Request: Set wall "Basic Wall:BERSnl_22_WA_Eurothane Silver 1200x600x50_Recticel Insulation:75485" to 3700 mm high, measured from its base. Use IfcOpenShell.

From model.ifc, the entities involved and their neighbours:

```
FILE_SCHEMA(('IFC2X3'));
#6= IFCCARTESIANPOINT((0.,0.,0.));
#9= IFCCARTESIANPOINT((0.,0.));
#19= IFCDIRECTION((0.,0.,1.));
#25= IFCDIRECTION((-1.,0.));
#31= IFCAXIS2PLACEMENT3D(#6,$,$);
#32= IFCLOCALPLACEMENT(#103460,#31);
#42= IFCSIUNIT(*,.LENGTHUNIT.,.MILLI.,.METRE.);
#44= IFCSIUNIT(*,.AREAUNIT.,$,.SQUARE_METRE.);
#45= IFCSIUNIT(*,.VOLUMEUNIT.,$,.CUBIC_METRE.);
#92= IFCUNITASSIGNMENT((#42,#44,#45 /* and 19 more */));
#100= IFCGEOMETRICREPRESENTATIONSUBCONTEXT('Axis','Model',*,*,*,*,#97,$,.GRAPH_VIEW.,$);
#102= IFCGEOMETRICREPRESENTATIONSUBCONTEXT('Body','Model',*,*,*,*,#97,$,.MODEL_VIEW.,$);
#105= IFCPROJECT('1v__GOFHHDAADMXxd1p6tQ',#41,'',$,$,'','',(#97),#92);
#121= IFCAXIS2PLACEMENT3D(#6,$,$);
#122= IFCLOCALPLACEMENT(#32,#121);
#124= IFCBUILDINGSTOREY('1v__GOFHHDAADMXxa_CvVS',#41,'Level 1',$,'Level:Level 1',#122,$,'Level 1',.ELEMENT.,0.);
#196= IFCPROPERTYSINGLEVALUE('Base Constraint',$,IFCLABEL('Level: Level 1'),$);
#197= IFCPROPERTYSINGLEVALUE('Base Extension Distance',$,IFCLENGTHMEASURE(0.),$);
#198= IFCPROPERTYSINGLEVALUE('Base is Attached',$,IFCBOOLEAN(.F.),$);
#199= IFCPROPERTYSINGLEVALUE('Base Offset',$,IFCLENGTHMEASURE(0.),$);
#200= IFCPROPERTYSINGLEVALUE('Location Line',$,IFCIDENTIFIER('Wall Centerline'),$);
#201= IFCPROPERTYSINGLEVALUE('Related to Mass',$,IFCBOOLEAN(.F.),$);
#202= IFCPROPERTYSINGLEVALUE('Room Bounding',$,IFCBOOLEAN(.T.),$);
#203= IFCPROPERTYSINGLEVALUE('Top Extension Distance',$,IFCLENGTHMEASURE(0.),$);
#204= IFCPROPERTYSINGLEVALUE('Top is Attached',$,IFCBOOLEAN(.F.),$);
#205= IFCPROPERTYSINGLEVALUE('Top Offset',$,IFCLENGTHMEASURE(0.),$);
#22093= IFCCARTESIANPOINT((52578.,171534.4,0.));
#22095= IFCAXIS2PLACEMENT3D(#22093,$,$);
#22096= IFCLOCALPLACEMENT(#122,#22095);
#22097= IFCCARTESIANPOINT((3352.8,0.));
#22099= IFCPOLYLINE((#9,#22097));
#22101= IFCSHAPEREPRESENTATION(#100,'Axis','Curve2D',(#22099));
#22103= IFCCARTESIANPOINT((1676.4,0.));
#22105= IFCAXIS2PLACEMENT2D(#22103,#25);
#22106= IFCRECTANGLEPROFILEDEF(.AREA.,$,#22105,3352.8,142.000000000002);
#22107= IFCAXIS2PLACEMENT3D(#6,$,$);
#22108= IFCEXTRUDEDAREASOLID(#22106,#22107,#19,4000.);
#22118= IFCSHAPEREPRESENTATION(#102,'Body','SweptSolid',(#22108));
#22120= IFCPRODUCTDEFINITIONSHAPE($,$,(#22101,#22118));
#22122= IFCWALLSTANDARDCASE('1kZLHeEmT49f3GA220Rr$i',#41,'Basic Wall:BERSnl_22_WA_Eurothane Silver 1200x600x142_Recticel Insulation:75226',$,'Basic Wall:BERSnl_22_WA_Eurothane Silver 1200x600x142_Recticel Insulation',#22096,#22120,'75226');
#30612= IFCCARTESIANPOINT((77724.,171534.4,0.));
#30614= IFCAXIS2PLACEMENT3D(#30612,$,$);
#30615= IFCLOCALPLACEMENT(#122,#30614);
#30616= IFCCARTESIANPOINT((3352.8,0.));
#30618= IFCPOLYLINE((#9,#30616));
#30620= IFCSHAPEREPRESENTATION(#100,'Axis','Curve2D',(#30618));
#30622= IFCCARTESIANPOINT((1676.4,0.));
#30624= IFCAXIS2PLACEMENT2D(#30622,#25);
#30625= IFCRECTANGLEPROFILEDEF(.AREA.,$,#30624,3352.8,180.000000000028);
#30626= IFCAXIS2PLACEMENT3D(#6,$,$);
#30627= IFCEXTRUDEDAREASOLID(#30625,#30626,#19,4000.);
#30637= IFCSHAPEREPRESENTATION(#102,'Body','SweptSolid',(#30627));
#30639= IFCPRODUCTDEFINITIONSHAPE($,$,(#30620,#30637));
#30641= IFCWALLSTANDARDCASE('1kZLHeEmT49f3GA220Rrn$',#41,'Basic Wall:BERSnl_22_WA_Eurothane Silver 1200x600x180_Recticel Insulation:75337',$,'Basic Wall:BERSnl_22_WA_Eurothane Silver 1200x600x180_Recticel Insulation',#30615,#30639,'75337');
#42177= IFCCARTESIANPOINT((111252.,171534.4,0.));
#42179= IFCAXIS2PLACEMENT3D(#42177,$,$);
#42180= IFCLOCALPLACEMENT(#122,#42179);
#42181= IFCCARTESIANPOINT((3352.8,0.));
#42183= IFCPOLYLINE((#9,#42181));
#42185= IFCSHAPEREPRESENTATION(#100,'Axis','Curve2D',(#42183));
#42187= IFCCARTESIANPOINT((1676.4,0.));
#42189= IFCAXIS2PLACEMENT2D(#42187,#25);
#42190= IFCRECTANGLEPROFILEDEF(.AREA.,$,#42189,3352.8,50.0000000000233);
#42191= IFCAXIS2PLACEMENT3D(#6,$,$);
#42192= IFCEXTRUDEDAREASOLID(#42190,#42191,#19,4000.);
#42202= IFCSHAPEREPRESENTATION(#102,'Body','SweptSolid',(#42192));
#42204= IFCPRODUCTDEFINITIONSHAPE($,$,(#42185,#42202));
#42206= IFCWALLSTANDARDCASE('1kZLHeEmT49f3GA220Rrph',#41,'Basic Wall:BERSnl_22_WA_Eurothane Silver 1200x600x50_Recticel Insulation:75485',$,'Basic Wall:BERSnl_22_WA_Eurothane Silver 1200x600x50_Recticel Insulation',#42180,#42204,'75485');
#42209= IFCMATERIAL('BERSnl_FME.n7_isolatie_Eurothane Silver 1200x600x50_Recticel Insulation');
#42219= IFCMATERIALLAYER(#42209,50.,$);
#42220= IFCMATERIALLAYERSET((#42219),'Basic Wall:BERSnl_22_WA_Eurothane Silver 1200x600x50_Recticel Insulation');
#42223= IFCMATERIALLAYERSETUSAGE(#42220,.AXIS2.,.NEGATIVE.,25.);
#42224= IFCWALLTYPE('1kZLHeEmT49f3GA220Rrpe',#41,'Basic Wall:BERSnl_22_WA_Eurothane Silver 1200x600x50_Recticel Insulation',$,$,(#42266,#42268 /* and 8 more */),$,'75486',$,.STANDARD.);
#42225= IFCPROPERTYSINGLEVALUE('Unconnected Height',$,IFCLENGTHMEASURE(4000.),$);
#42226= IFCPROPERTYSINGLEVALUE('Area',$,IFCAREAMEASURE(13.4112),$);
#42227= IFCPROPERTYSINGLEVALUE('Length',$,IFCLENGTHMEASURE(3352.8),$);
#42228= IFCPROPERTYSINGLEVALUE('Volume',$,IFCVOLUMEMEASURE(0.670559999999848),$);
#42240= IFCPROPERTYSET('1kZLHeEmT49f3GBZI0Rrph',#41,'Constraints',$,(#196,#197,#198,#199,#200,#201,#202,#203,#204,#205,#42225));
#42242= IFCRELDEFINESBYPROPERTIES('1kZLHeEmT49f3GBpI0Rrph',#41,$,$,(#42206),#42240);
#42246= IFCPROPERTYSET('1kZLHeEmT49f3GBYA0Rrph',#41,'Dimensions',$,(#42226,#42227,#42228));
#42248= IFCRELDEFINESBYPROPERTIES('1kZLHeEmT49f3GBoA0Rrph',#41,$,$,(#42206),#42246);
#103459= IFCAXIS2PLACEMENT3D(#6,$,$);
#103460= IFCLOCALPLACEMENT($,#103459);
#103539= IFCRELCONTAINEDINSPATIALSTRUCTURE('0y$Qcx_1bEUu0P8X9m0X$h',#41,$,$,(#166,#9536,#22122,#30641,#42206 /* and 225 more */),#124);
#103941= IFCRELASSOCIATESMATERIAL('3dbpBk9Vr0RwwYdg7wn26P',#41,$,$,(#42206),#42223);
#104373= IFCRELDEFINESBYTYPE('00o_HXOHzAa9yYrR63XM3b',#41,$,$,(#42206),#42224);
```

```python
import ifcopenshell
import ifcopenshell.api.pset
import ifcopenshell.geom
import ifcopenshell.util.element
import ifcopenshell.util.representation
import ifcopenshell.util.shape
import ifcopenshell.util.unit

model = ifcopenshell.open("model.ifc")
area_scale = ifcopenshell.util.unit.calculate_unit_scale(model, "AREAUNIT")
volume_scale = ifcopenshell.util.unit.calculate_unit_scale(model, "VOLUMEUNIT")
settings = ifcopenshell.geom.settings()


def volume(element):
    """Net volume in cubic metres, openings subtracted."""
    shape = ifcopenshell.geom.create_shape(settings, element)
    return ifcopenshell.util.shape.get_volume(shape.geometry)


wall = model.by_guid("1kZLHeEmT49f3GA220Rrph")
before = volume(wall)

body = ifcopenshell.util.representation.get_representation(wall, "Model", "Body")
solid = body.Items[0]
old_height = solid.Depth
solid.Depth = 3700.0
after = volume(wall)
thickness = 0.05  # wall thickness in metres

# Update the stored height, areas and volumes.
pset = model.by_id(ifcopenshell.util.element.get_pset(wall, "Constraints", should_inherit=False)["id"])
ifcopenshell.api.pset.edit_pset(model, pset=pset, properties={
    "Unconnected Height": model.create_entity("IfcLengthMeasure", solid.Depth),
})
pset = model.by_id(ifcopenshell.util.element.get_pset(wall, "Dimensions", should_inherit=False)["id"])
ifcopenshell.api.pset.edit_pset(model, pset=pset, properties={
    "Area": model.create_entity("IfcAreaMeasure", after / thickness / area_scale),
    "Volume": model.create_entity("IfcVolumeMeasure", after / volume_scale),
})

print(f"height {old_height:g} -> {solid.Depth:g}, volume {before:.3f} -> {after:.3f} m3")

model.write("model_v2.ifc")
```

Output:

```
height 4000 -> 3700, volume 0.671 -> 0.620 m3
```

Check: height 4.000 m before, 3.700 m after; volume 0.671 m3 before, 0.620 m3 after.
